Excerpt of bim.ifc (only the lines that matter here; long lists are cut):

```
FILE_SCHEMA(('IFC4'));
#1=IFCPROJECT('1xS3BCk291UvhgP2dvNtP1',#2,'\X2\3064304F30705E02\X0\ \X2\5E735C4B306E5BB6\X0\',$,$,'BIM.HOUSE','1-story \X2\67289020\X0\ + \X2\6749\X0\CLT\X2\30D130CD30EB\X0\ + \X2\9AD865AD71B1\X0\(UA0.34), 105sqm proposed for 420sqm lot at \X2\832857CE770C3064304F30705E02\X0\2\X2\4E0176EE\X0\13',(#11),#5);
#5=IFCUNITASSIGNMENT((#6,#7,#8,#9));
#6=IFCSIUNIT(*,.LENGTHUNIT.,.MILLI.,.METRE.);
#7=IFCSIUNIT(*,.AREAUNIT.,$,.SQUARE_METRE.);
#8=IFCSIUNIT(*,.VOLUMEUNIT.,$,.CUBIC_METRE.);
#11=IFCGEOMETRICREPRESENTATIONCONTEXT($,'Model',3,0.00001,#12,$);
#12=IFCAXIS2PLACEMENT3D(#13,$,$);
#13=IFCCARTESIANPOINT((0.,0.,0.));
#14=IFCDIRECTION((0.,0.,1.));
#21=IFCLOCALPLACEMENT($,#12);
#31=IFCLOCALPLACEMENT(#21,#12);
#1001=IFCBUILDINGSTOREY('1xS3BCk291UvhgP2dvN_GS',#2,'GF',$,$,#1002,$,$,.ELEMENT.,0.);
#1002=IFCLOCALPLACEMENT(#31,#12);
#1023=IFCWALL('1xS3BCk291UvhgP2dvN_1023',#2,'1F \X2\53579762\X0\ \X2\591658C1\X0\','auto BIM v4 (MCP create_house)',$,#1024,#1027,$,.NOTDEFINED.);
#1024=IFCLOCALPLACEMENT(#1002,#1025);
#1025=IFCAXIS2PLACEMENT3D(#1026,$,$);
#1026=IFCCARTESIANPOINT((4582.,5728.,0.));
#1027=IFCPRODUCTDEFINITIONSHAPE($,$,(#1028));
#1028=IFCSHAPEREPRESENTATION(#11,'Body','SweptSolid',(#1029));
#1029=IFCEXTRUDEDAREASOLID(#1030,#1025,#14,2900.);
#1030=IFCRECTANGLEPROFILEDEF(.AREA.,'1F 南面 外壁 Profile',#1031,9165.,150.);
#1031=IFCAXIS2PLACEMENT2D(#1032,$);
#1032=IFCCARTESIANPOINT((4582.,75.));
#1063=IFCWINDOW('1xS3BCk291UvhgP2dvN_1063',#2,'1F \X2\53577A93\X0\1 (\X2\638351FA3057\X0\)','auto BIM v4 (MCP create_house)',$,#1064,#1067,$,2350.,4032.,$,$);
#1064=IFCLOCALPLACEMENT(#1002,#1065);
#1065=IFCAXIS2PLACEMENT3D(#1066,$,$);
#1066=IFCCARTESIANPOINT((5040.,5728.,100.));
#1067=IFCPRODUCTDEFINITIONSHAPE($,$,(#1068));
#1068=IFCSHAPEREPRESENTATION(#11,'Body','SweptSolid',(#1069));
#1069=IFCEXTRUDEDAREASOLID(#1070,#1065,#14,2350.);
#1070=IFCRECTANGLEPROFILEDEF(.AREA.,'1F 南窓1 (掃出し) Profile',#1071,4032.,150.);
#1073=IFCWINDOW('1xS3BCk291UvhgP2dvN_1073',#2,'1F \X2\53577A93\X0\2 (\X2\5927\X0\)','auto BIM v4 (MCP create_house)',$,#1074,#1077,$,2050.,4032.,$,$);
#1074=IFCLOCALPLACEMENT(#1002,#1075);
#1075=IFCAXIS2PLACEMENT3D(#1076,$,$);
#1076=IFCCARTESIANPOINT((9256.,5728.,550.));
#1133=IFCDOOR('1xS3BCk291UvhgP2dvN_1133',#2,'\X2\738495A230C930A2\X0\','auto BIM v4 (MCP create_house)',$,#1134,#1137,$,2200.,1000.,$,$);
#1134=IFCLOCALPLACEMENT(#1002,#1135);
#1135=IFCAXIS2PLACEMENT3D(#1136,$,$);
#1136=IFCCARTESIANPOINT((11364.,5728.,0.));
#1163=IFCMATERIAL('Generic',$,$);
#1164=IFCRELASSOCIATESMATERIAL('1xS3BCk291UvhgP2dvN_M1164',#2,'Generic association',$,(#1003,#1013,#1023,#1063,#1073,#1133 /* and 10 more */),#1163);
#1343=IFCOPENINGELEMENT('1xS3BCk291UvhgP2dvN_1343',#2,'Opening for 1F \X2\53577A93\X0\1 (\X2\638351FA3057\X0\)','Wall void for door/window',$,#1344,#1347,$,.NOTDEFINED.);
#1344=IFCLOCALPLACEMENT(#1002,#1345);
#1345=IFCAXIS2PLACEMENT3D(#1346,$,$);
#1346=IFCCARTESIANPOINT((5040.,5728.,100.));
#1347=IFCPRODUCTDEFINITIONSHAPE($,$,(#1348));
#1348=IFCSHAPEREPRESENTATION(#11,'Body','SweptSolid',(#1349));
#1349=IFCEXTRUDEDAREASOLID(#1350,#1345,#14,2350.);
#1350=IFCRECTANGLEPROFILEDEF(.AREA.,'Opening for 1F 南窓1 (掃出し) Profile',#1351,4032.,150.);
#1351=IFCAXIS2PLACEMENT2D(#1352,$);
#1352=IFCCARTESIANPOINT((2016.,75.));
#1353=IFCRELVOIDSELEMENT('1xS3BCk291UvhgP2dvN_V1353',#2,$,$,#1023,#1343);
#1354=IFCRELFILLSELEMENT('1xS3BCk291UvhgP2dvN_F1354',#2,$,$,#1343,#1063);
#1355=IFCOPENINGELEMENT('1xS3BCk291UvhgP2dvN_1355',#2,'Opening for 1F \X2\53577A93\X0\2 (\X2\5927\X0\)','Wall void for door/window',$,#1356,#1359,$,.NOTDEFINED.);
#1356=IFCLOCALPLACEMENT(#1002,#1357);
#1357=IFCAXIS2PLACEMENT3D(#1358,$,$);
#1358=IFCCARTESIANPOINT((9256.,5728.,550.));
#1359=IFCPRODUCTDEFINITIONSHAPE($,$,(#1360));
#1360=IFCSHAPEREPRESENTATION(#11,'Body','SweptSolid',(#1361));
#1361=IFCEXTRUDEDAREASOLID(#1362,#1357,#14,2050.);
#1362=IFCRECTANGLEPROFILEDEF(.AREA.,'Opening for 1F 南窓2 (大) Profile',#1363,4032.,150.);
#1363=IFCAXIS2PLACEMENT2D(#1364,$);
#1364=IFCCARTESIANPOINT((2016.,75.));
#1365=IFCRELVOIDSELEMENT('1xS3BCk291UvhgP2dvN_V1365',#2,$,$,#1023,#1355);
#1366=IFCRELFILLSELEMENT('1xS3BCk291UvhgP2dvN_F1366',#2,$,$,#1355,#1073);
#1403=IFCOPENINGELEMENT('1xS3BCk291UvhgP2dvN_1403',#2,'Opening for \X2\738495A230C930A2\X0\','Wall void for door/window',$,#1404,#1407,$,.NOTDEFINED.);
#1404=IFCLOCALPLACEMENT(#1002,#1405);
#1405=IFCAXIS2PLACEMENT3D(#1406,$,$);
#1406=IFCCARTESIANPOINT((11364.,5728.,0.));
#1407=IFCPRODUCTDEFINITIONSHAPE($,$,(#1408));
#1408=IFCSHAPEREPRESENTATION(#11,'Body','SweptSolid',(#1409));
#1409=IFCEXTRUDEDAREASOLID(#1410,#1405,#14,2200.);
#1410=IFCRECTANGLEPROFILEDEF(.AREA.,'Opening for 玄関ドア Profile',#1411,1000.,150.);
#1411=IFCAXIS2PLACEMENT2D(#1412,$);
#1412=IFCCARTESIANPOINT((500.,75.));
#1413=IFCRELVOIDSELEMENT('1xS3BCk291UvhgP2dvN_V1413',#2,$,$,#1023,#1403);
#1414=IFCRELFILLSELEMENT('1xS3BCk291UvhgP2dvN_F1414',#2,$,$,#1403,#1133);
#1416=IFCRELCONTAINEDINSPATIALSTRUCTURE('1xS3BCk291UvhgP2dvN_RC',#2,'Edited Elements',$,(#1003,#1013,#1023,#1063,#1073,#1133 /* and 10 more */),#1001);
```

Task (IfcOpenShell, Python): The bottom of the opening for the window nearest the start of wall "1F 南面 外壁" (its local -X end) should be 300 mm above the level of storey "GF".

```python
import numpy as np
import ifcopenshell
import ifcopenshell.api.geometry
import ifcopenshell.geom
import ifcopenshell.util.element
import ifcopenshell.util.placement
import ifcopenshell.util.shape
import ifcopenshell.util.unit

model = ifcopenshell.open("bim.ifc")
unit_scale = ifcopenshell.util.unit.calculate_unit_scale(model)

window = model.by_id(1063)
opening = window.FillsVoids[0].RelatingOpeningElement
storey = ifcopenshell.util.element.get_container(window, ifc_class="IfcBuildingStorey")
level = ifcopenshell.util.placement.get_local_placement(storey.ObjectPlacement)[2, 3]

# The opening's origin need not be at the sill, so measure its lowest point.
shape = ifcopenshell.geom.create_shape(ifcopenshell.geom.settings(), opening)
bottom = ifcopenshell.util.shape.get_shape_bottom_elevation(shape, shape.geometry) / unit_scale
dz = level + 300.0 - bottom

shift = np.array([0.0, 0.0, dz])
# The window is not placed relative to its opening, so move both.
for product in (opening, window):
    matrix = ifcopenshell.util.placement.get_local_placement(product.ObjectPlacement)
    matrix[:3, 3] += shift
    ifcopenshell.api.geometry.edit_object_placement(model, product=product, matrix=matrix, is_si=False)

print(f"moved by {dz * unit_scale:+.3f} m")

model.write("bim_updated.ifc")
```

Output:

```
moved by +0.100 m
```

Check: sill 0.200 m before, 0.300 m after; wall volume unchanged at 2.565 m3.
